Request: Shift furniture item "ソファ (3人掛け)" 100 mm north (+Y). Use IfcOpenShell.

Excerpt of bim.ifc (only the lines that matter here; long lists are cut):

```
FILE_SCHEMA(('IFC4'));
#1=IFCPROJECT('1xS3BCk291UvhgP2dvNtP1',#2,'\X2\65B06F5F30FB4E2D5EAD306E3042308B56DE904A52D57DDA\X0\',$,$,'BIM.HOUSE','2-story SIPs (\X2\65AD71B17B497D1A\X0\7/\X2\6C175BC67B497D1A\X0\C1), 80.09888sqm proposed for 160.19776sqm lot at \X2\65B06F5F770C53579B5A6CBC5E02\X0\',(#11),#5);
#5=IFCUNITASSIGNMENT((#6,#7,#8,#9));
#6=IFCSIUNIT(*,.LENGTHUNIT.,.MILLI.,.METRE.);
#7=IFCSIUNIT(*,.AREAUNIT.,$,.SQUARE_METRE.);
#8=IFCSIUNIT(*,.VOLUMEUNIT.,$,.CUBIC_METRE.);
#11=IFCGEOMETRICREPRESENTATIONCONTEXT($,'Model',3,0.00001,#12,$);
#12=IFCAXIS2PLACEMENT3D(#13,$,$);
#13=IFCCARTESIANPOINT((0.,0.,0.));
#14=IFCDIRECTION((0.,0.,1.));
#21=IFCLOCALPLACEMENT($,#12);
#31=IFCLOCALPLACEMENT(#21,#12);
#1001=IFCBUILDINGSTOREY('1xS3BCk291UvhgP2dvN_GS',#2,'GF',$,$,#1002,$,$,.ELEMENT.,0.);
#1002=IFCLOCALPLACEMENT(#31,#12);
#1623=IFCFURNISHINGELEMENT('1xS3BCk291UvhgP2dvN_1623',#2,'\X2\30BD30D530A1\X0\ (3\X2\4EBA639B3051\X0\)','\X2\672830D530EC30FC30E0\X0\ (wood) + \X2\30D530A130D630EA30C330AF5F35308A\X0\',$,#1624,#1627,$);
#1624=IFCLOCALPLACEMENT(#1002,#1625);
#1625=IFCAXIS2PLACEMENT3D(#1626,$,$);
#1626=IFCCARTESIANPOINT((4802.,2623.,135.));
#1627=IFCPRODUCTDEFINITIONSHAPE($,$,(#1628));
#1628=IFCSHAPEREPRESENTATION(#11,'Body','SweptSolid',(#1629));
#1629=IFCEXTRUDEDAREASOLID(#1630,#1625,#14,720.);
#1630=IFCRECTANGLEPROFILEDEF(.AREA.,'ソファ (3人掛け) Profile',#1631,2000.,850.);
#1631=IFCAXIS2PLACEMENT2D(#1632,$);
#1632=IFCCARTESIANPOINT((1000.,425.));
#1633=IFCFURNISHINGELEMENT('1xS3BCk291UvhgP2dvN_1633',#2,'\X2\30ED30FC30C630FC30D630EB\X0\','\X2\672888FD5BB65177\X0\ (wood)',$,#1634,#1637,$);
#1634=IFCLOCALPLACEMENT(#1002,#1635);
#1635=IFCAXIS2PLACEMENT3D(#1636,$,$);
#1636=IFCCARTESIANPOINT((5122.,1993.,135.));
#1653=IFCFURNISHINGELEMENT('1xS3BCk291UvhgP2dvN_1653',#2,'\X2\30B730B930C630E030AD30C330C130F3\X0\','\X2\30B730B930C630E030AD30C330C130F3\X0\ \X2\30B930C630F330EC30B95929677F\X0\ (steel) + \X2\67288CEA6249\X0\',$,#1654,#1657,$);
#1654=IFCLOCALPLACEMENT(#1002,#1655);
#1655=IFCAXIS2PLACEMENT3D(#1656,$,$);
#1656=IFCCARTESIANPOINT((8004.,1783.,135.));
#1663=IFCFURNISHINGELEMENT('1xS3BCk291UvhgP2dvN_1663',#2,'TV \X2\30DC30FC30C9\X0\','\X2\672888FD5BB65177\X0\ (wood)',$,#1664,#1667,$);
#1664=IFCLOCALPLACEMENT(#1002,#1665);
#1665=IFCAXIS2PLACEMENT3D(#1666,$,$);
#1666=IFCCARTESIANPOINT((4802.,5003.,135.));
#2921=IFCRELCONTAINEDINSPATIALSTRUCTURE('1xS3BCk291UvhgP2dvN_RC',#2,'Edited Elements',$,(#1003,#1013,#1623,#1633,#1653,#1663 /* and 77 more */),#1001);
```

```python
import ifcopenshell
import ifcopenshell.api.geometry
import ifcopenshell.util.placement
import ifcopenshell.util.unit

model = ifcopenshell.open("bim.ifc")
unit_scale = ifcopenshell.util.unit.calculate_unit_scale(model)

item = model.by_id(1623)
matrix = ifcopenshell.util.placement.get_local_placement(item.ObjectPlacement)
matrix[1, 3] += 0.1 / unit_scale
ifcopenshell.api.geometry.edit_object_placement(model, product=item, matrix=matrix, is_si=False)

print(ifcopenshell.util.placement.get_local_placement(item.ObjectPlacement).round(3) + 0.0)

model.write("bim_v2.ifc")
```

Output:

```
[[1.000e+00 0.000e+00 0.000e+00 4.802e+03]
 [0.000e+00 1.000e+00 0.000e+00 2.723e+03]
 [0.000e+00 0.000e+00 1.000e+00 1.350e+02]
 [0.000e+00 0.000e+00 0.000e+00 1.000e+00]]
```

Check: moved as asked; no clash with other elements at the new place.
